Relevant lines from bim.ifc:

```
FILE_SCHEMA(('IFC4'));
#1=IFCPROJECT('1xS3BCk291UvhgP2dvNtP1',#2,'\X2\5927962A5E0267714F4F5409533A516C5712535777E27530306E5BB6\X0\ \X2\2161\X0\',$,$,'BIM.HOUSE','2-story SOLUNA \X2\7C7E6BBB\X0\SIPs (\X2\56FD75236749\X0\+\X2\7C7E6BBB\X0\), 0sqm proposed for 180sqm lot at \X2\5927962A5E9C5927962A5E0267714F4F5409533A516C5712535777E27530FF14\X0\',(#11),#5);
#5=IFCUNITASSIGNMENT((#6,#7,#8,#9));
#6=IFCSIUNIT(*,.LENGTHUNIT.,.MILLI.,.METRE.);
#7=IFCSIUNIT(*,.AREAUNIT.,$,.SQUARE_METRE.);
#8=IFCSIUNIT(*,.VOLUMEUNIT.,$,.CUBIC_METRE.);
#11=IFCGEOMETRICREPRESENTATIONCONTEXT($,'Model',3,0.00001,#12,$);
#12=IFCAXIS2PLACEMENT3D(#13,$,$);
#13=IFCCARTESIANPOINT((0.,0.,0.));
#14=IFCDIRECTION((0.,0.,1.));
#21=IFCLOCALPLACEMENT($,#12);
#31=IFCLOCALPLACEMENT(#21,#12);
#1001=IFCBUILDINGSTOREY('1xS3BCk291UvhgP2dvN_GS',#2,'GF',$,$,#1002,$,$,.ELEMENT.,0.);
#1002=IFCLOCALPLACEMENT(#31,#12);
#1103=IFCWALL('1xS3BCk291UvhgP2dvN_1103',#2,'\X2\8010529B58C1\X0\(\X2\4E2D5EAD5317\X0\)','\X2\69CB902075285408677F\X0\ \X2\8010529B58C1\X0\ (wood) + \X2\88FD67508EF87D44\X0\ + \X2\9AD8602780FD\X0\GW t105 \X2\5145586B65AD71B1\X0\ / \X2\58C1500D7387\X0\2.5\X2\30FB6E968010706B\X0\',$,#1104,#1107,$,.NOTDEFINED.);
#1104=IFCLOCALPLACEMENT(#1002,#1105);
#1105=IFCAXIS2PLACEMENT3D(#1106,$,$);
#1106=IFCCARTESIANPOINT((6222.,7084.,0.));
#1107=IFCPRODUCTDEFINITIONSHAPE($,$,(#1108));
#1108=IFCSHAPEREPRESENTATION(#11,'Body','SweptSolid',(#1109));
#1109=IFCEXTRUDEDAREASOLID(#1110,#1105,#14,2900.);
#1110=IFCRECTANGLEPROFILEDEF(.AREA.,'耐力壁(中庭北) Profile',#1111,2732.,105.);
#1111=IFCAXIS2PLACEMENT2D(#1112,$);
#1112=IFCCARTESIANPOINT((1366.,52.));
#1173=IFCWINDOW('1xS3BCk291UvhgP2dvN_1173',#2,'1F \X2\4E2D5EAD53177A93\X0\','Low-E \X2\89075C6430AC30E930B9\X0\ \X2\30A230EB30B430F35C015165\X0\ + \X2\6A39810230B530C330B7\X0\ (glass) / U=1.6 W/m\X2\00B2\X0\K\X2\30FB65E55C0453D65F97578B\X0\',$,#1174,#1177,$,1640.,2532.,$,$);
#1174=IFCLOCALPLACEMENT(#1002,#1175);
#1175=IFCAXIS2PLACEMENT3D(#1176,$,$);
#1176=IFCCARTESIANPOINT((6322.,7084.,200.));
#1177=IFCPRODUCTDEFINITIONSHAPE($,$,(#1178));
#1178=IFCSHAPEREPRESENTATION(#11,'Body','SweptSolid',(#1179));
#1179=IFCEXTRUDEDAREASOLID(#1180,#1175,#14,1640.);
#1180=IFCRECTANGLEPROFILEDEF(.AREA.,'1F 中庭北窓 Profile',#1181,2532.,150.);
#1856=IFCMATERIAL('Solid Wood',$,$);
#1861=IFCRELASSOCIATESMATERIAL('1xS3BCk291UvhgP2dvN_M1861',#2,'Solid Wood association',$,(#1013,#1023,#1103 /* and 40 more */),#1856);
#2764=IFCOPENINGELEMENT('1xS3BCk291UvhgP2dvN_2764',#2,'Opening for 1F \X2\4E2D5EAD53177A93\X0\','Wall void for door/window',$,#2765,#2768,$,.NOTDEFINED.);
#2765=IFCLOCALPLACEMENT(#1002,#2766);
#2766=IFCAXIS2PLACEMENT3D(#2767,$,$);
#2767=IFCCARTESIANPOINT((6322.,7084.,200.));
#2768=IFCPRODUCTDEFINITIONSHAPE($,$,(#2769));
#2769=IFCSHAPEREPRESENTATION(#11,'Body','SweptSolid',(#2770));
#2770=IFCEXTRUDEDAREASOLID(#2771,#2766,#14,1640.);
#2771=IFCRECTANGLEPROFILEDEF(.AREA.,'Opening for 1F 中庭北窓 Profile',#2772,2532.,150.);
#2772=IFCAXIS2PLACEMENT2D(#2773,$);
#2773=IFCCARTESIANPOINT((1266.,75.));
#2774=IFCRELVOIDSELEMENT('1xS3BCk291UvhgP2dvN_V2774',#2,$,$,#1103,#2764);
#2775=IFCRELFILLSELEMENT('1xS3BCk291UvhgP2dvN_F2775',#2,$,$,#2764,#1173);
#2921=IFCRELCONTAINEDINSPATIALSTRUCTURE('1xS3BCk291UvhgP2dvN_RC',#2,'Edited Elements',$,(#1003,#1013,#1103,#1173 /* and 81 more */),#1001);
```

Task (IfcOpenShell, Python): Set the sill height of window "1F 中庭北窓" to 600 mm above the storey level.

```python
import numpy as np
import ifcopenshell
import ifcopenshell.api.geometry
import ifcopenshell.geom
import ifcopenshell.util.element
import ifcopenshell.util.placement
import ifcopenshell.util.shape
import ifcopenshell.util.unit

model = ifcopenshell.open("bim.ifc")
unit_scale = ifcopenshell.util.unit.calculate_unit_scale(model)

window = model.by_id(1173)
opening = window.FillsVoids[0].RelatingOpeningElement
storey = ifcopenshell.util.element.get_container(window, ifc_class="IfcBuildingStorey")
level = ifcopenshell.util.placement.get_local_placement(storey.ObjectPlacement)[2, 3]

# The opening's origin need not be at the sill, so measure its lowest point.
shape = ifcopenshell.geom.create_shape(ifcopenshell.geom.settings(), opening)
bottom = ifcopenshell.util.shape.get_shape_bottom_elevation(shape, shape.geometry) / unit_scale
dz = level + 600.0 - bottom

shift = np.array([0.0, 0.0, dz])
# The window is not placed relative to its opening, so move both.
for product in (opening, window):
    matrix = ifcopenshell.util.placement.get_local_placement(product.ObjectPlacement)
    matrix[:3, 3] += shift
    ifcopenshell.api.geometry.edit_object_placement(model, product=product, matrix=matrix, is_si=False)

print(f"moved by {dz * unit_scale:+.3f} m")

model.write("bim-out.ifc")
```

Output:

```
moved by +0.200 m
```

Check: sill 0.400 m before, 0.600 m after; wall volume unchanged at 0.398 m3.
